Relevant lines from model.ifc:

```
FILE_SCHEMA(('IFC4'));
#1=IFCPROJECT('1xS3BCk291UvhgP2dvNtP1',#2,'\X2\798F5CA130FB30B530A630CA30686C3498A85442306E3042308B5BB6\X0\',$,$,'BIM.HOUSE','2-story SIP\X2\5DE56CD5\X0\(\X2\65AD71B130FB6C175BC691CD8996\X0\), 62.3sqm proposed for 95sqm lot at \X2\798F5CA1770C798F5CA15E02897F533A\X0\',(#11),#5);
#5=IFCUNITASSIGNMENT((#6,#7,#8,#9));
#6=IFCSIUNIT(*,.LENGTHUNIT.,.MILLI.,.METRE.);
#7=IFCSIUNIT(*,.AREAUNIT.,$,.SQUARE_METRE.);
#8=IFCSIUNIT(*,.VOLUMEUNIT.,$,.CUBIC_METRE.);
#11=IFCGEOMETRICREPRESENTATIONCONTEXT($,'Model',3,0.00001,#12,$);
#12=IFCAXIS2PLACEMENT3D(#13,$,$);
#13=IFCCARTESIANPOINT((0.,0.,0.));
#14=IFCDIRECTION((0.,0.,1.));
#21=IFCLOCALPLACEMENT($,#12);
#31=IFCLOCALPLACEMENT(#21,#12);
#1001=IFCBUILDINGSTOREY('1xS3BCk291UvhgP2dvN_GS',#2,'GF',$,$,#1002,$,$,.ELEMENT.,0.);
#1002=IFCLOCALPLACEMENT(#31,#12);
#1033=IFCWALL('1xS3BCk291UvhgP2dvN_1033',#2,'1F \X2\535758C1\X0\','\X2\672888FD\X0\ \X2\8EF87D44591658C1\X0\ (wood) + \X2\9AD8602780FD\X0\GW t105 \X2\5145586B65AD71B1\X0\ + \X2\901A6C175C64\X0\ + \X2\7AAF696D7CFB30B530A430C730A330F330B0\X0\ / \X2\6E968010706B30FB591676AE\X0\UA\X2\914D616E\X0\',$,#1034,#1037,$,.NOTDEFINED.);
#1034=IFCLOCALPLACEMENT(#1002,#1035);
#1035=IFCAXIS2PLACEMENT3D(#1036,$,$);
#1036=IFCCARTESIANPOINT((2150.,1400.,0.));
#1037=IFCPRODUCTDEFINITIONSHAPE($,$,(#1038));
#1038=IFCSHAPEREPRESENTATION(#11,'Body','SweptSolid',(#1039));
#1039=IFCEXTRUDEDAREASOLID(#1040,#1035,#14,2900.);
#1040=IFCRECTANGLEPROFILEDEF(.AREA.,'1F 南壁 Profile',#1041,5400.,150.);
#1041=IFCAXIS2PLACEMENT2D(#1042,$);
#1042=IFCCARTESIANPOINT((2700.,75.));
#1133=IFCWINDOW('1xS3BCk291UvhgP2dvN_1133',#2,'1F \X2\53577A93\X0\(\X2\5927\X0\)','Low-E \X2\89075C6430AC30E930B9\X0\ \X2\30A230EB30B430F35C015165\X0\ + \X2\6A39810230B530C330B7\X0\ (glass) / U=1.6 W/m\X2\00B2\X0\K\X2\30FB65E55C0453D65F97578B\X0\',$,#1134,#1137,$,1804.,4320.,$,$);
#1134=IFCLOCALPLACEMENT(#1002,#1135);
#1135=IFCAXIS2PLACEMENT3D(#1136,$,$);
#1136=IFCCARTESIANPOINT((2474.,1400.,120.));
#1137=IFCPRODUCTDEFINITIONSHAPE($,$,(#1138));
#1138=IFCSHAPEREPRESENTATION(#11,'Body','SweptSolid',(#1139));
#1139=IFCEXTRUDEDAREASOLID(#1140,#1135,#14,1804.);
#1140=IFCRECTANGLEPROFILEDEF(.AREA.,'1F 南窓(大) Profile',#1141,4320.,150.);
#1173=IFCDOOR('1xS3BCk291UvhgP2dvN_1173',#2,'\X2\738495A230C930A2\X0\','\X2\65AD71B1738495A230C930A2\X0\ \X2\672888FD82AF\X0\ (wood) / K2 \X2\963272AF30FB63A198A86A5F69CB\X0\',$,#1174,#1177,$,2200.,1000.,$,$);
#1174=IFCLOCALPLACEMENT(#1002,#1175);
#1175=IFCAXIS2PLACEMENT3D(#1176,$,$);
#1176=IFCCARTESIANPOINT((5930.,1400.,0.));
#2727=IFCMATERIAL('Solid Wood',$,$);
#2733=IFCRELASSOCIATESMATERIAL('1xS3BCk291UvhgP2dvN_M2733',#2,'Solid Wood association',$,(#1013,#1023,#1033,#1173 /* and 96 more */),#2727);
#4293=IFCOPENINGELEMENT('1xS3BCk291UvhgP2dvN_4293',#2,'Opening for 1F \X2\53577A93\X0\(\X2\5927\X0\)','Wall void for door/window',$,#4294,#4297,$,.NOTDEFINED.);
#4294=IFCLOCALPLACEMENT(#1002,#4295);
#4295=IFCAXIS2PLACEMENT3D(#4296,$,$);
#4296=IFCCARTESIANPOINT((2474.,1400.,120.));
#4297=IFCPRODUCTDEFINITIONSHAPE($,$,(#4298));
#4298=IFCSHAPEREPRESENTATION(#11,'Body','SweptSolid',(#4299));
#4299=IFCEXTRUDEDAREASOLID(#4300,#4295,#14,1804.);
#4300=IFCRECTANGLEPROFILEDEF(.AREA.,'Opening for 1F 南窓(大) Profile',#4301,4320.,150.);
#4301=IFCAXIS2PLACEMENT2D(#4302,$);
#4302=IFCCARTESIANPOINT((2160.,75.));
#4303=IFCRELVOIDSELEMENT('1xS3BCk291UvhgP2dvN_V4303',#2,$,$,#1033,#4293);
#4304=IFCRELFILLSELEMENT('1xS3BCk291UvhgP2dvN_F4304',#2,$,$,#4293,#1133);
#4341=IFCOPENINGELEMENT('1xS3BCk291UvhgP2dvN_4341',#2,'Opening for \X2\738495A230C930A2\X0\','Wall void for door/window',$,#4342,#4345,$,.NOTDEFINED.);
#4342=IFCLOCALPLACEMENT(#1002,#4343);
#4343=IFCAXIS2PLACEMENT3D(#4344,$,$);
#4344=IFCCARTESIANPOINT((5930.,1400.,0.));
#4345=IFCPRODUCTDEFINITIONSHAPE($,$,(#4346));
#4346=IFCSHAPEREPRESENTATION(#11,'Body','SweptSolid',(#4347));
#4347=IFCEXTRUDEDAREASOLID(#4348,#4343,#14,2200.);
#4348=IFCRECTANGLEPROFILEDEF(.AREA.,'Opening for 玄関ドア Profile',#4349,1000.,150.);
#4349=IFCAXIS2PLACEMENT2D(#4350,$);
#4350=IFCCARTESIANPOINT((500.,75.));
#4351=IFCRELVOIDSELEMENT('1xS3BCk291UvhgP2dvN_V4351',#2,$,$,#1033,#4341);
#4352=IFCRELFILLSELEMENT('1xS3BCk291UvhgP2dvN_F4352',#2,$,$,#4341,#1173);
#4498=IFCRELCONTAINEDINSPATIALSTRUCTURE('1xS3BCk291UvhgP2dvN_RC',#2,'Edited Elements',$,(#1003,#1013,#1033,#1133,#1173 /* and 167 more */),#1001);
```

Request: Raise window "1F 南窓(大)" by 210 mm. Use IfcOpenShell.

```python
import numpy as np
import ifcopenshell
import ifcopenshell.api.geometry
import ifcopenshell.util.placement
import ifcopenshell.util.unit

model = ifcopenshell.open("model.ifc")
unit_scale = ifcopenshell.util.unit.calculate_unit_scale(model)

window = model.by_guid("1xS3BCk291UvhgP2dvN_1133")
opening = window.FillsVoids[0].RelatingOpeningElement
dz = 0.21 / unit_scale

shift = np.array([0.0, 0.0, dz])
# The window is not placed relative to its opening, so move both.
for product in (opening, window):
    matrix = ifcopenshell.util.placement.get_local_placement(product.ObjectPlacement)
    matrix[:3, 3] += shift
    ifcopenshell.api.geometry.edit_object_placement(model, product=product, matrix=matrix, is_si=False)

print(f"moved by {dz * unit_scale:+.3f} m")

model.write("model_rev.ifc")
```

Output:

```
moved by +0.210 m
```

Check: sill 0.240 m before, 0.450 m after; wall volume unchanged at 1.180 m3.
